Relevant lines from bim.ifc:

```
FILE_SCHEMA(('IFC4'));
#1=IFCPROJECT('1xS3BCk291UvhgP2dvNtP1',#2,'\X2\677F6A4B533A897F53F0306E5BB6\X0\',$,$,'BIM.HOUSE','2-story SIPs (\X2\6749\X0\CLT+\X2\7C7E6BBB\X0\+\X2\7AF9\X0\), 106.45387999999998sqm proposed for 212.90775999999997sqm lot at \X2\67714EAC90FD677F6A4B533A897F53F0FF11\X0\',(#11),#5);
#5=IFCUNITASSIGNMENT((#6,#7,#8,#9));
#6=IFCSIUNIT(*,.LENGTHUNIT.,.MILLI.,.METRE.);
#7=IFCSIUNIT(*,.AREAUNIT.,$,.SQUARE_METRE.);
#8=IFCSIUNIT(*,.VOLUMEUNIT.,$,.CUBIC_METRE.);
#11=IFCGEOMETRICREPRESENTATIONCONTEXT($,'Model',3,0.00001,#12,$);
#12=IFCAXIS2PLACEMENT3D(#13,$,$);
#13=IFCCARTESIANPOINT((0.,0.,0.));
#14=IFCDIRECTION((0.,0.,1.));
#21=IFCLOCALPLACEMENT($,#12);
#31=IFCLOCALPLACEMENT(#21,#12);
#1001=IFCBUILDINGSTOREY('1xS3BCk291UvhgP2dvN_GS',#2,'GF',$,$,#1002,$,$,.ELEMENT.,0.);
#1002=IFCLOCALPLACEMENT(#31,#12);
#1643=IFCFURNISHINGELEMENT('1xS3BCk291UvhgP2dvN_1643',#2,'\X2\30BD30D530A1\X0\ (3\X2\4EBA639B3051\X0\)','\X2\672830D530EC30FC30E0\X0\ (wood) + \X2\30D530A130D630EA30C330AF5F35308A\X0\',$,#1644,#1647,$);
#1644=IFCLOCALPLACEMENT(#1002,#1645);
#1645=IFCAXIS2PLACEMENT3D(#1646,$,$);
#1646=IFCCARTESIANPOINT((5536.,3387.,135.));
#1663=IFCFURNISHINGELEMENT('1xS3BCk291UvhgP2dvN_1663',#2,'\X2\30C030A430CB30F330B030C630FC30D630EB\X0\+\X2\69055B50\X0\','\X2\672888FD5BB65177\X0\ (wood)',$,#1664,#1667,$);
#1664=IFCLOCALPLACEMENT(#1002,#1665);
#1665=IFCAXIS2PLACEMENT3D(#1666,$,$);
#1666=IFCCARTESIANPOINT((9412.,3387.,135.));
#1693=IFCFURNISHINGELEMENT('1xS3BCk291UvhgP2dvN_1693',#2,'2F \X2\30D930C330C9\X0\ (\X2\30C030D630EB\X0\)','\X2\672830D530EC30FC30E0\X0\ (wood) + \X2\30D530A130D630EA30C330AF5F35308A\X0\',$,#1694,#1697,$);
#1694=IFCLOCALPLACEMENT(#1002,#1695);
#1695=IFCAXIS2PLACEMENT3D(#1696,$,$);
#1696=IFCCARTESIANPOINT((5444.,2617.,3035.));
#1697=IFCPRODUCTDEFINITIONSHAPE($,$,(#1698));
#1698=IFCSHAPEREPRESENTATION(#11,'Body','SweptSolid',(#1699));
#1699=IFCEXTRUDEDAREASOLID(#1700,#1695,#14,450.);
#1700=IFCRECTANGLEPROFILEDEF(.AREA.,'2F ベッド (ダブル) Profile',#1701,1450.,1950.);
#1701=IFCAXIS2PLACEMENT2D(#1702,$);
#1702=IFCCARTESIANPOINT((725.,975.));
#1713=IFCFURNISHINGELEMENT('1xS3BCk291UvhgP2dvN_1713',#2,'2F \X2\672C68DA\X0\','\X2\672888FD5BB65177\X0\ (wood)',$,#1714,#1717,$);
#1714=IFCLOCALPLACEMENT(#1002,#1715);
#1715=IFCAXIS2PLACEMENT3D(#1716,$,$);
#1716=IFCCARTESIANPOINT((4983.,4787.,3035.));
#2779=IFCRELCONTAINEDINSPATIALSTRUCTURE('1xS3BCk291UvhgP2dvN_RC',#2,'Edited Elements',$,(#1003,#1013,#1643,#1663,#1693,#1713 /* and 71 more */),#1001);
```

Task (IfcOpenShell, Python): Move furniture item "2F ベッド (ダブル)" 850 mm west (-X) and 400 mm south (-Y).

```python
import ifcopenshell
import ifcopenshell.api.geometry
import ifcopenshell.util.placement

model = ifcopenshell.open("bim.ifc")

item = model.by_guid("1xS3BCk291UvhgP2dvN_1693")
matrix = ifcopenshell.util.placement.get_local_placement(item.ObjectPlacement)
matrix[0, 3] -= 850.0
matrix[1, 3] -= 400.0
ifcopenshell.api.geometry.edit_object_placement(model, product=item, matrix=matrix, is_si=False)

print(ifcopenshell.util.placement.get_local_placement(item.ObjectPlacement).round(3) + 0.0)

model.write("bim_edited.ifc")
```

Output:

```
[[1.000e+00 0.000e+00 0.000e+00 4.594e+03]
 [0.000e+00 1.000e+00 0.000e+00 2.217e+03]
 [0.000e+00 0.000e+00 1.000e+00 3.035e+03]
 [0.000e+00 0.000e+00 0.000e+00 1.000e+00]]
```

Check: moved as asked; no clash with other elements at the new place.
